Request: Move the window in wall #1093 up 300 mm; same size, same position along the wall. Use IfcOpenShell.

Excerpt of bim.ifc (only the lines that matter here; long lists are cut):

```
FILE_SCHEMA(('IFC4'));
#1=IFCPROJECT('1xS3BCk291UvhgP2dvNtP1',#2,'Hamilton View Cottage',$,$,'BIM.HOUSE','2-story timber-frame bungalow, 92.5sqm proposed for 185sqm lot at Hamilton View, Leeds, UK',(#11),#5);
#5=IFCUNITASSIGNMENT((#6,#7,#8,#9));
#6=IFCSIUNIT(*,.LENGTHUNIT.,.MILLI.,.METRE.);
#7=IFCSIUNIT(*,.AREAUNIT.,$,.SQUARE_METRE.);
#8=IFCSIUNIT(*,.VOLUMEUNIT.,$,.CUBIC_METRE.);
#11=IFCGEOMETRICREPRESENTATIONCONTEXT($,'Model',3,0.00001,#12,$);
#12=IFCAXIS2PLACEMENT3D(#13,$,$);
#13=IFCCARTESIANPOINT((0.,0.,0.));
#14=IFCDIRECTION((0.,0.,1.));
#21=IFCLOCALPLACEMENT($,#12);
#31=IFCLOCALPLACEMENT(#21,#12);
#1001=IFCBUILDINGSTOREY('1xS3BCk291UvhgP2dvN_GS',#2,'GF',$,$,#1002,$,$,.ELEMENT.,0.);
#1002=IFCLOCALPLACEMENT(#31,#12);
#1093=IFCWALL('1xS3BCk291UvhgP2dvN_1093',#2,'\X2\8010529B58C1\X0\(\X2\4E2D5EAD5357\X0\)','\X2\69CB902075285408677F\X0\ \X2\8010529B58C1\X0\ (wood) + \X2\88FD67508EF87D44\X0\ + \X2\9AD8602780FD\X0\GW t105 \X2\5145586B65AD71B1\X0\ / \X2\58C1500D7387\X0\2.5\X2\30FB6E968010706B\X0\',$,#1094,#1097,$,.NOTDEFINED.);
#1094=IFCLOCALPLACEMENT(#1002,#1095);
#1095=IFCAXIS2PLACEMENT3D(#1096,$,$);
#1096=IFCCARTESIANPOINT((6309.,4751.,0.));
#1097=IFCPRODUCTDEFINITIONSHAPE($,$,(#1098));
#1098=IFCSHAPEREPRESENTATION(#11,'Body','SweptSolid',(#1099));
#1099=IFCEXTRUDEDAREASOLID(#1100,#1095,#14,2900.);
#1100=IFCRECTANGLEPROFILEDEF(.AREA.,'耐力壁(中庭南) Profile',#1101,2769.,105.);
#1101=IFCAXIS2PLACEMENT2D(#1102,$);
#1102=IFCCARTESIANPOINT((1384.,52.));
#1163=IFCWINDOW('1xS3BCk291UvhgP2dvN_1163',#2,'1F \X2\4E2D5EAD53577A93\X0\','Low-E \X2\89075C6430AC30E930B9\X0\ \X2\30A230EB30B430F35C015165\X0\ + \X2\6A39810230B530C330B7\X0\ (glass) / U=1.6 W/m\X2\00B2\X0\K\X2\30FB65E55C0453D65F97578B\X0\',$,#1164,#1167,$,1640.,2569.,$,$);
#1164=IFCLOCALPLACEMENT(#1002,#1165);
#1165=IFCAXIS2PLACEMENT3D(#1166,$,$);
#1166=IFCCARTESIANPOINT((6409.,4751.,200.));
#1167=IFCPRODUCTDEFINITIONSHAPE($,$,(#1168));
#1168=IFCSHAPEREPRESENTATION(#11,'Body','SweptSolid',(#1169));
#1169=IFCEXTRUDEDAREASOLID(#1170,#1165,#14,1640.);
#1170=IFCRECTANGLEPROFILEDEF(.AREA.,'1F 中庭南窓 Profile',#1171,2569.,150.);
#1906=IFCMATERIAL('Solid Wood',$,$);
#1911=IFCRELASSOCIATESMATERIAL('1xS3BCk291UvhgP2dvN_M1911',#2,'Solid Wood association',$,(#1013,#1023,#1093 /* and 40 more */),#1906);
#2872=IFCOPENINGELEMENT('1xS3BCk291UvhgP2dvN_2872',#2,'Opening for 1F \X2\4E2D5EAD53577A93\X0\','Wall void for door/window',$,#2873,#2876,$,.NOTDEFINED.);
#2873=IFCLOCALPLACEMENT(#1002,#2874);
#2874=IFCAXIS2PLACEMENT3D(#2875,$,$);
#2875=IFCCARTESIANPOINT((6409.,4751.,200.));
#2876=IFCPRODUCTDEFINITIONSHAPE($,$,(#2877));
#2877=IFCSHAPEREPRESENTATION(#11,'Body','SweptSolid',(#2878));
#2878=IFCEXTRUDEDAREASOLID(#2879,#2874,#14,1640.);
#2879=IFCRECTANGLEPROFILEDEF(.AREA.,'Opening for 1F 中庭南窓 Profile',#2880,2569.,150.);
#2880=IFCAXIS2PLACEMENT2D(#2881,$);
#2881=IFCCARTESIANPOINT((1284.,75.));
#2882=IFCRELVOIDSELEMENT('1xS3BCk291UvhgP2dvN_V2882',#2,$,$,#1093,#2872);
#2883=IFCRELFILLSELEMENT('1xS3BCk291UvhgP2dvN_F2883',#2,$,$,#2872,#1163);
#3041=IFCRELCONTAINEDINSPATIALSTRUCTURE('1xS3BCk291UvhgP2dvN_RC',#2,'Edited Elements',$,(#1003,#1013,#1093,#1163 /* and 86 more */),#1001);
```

```python
import numpy as np
import ifcopenshell
import ifcopenshell.api.geometry
import ifcopenshell.util.placement
import ifcopenshell.util.unit

model = ifcopenshell.open("bim.ifc")
unit_scale = ifcopenshell.util.unit.calculate_unit_scale(model)

window = model.by_guid("1xS3BCk291UvhgP2dvN_1163")
opening = window.FillsVoids[0].RelatingOpeningElement
dz = 0.3 / unit_scale

shift = np.array([0.0, 0.0, dz])
# The window is not placed relative to its opening, so move both.
for product in (opening, window):
    matrix = ifcopenshell.util.placement.get_local_placement(product.ObjectPlacement)
    matrix[:3, 3] += shift
    ifcopenshell.api.geometry.edit_object_placement(model, product=product, matrix=matrix, is_si=False)

print(f"moved by {dz * unit_scale:+.3f} m")

model.write("bim_rev.ifc")
```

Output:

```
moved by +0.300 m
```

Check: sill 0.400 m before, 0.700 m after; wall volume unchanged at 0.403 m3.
